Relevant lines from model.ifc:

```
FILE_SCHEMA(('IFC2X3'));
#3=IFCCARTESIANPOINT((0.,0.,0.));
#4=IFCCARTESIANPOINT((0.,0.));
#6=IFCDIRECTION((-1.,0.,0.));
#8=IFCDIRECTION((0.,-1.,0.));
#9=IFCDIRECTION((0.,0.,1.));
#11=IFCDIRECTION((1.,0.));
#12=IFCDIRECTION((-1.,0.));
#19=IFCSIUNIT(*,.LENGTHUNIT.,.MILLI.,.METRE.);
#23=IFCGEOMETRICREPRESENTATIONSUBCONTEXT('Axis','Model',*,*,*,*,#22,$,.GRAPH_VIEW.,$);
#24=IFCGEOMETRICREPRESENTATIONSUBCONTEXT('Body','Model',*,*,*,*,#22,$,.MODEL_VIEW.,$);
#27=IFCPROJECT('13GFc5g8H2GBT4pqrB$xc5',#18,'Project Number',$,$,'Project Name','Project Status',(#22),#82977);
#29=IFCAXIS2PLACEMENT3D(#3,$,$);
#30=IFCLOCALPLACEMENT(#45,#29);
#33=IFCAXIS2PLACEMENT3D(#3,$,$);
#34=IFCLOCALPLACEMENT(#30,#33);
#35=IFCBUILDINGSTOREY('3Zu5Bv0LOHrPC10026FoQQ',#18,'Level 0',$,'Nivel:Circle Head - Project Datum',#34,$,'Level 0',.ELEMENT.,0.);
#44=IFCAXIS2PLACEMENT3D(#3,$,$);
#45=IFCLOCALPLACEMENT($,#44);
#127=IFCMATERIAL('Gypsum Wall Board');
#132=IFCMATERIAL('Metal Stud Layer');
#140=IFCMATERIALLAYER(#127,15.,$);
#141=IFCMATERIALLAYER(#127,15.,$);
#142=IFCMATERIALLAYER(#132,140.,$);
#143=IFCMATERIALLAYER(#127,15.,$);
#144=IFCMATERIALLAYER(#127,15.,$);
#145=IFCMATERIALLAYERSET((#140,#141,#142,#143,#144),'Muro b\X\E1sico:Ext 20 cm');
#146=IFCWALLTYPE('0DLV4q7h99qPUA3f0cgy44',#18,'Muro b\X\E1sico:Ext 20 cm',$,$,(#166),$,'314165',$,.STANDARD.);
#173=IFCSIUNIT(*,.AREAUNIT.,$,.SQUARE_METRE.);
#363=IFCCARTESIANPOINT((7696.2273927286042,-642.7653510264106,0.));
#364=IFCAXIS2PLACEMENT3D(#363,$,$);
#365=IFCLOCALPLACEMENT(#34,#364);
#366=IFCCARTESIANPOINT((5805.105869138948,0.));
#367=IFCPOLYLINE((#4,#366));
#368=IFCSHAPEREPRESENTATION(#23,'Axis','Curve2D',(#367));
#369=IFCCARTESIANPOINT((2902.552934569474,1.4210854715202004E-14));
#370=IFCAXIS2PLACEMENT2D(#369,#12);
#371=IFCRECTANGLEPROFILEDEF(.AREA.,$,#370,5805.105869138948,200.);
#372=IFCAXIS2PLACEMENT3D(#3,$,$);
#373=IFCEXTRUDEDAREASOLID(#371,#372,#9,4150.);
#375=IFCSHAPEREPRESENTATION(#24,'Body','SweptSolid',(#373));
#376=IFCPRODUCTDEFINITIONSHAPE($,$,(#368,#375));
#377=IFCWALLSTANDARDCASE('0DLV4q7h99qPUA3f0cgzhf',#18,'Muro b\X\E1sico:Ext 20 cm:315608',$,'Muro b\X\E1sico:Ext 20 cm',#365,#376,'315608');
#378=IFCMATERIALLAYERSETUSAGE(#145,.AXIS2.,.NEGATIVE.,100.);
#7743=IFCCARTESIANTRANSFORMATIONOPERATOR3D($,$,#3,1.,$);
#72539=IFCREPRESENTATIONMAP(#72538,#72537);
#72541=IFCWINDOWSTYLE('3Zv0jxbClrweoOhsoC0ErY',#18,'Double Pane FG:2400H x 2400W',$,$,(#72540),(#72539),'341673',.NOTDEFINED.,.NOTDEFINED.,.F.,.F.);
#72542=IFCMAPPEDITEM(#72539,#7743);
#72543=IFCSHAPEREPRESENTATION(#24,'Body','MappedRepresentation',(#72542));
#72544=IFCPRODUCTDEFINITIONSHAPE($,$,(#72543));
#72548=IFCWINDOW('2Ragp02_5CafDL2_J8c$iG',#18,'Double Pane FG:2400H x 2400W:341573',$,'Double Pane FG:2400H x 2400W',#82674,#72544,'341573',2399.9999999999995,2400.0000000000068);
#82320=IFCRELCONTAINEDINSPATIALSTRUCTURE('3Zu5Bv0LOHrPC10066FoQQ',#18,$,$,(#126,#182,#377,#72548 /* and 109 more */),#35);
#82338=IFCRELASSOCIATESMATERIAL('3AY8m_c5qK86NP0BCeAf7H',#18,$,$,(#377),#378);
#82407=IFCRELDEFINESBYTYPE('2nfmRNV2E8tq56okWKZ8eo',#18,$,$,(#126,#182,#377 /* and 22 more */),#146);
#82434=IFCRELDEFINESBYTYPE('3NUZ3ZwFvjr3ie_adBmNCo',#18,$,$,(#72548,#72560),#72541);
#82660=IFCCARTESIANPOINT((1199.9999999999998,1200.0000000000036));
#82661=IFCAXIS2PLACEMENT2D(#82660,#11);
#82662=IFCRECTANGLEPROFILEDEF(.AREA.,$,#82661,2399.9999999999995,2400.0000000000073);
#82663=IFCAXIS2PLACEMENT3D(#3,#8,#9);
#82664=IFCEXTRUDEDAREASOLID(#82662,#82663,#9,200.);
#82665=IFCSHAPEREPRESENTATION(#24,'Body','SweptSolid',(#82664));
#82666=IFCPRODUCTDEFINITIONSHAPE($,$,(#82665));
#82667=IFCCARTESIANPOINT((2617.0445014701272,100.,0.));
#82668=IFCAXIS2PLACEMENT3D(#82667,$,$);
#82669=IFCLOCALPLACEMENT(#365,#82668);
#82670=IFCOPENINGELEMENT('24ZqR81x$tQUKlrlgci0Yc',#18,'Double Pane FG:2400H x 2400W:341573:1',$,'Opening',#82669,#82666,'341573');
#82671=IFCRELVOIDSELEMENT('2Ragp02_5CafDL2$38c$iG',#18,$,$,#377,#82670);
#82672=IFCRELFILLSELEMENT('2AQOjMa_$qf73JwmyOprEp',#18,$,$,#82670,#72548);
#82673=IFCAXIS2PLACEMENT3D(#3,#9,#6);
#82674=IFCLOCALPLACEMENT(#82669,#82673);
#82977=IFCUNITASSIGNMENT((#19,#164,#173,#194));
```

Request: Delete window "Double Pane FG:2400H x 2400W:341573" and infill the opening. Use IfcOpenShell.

```python
import ifcopenshell
import ifcopenshell.api.feature
import ifcopenshell.api.root
import ifcopenshell.geom
import ifcopenshell.util.shape

model = ifcopenshell.open("model.ifc")
settings = ifcopenshell.geom.settings()


def volume(element):
    """Net volume in cubic metres, openings subtracted."""
    shape = ifcopenshell.geom.create_shape(settings, element)
    return ifcopenshell.util.shape.get_volume(shape.geometry)


window = model.by_guid("2Ragp02_5CafDL2_J8c$iG")
opening = window.FillsVoids[0].RelatingOpeningElement
wall = opening.VoidsElements[0].RelatingBuildingElement
before = volume(wall)

ifcopenshell.api.root.remove_product(model, product=window)
ifcopenshell.api.feature.remove_feature(model, feature=opening)

after = volume(wall)

print(f"wall volume {before:.3f} -> {after:.3f} m3")

model.write("model-out.ifc")
```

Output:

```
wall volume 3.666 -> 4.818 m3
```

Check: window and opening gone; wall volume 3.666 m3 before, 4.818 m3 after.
